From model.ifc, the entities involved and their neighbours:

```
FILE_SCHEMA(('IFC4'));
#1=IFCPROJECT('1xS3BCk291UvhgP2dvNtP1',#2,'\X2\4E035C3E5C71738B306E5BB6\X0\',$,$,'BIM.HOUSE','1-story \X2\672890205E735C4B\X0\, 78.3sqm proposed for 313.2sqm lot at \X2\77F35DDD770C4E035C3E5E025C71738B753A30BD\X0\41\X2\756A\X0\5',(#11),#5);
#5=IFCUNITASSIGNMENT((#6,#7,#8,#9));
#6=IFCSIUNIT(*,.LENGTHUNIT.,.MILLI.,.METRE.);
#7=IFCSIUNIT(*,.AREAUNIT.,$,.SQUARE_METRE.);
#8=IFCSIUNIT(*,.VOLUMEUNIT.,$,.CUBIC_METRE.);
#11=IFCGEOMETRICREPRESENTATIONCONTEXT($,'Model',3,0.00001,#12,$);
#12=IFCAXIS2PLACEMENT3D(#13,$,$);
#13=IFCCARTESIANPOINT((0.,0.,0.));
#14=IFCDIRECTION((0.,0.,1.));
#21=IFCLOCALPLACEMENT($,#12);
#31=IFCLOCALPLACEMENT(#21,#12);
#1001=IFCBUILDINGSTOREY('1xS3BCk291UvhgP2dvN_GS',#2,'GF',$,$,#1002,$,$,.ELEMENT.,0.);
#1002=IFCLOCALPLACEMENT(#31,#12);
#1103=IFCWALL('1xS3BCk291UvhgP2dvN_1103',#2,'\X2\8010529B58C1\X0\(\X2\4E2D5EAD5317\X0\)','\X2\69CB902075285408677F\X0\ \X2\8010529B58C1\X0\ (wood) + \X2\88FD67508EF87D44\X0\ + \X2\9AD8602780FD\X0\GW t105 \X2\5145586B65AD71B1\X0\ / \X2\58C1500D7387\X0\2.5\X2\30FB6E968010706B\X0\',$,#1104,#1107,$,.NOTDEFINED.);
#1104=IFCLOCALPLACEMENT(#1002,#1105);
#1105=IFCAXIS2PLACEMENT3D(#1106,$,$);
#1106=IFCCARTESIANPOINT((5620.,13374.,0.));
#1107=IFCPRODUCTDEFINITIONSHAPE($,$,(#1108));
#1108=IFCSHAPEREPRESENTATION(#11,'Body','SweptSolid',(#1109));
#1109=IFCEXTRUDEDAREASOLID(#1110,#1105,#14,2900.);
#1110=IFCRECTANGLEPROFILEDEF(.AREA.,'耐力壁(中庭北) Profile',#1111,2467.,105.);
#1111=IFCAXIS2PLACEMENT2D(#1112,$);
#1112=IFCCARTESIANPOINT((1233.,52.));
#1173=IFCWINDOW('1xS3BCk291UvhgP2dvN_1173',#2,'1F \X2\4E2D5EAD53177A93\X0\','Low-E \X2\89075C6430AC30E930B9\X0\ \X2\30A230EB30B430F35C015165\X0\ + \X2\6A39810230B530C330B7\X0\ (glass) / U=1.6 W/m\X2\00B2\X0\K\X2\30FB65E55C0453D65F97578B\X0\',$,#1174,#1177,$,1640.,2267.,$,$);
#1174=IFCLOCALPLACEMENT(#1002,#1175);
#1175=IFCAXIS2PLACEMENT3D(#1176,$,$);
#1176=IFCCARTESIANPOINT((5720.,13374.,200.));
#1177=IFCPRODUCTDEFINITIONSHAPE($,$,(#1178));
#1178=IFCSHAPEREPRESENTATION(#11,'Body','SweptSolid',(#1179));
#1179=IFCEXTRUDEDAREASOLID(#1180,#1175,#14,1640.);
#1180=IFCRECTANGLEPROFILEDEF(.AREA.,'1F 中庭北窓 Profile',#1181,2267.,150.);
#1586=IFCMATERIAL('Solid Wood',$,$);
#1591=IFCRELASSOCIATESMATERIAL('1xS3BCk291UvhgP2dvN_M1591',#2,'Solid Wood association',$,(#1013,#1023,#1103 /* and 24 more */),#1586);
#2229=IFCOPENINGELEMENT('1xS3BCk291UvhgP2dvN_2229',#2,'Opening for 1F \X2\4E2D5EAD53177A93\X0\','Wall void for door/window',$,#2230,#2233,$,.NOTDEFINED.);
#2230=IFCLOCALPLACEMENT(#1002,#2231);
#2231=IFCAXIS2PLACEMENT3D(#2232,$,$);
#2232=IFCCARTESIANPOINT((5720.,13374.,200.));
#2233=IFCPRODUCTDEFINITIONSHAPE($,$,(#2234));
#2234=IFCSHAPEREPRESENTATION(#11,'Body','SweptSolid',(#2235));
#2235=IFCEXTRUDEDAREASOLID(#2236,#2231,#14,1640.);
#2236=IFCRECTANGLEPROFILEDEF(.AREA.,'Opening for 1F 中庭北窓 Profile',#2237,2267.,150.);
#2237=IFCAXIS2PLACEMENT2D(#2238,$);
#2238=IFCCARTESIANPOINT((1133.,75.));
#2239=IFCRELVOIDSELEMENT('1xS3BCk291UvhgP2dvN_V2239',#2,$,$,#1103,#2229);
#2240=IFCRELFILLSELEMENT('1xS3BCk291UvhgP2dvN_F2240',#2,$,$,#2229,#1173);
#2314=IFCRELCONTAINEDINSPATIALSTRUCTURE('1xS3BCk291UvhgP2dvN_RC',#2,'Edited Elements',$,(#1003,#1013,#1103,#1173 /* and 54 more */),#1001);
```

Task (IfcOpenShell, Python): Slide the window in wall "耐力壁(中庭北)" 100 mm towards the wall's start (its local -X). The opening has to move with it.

```python
import ifcopenshell
import ifcopenshell.api.geometry
import ifcopenshell.util.placement
import ifcopenshell.util.unit

model = ifcopenshell.open("model.ifc")
unit_scale = ifcopenshell.util.unit.calculate_unit_scale(model)

window = model.by_guid("1xS3BCk291UvhgP2dvN_1173")
opening = window.FillsVoids[0].RelatingOpeningElement
wall = opening.VoidsElements[0].RelatingBuildingElement

wall_matrix = ifcopenshell.util.placement.get_local_placement(wall.ObjectPlacement)
shift = wall_matrix[:3, 0] * -0.1 / unit_scale
before = ifcopenshell.util.placement.get_local_placement(window.ObjectPlacement)[:3, 3].copy()

# The window is not placed relative to its opening, so move both.
for product in (opening, window):
    matrix = ifcopenshell.util.placement.get_local_placement(product.ObjectPlacement)
    matrix[:3, 3] += shift
    ifcopenshell.api.geometry.edit_object_placement(model, product=product, matrix=matrix, is_si=False)

after = ifcopenshell.util.placement.get_local_placement(window.ObjectPlacement)[:3, 3]
print("window moved by", (after - before).round(3) + 0.0)

model.write("model_updated.ifc")
```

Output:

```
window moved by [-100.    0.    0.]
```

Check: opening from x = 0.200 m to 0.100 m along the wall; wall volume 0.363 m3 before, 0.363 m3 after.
